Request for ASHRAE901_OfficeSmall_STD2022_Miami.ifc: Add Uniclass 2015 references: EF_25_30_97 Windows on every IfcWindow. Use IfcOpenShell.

First a look at what the model holds.

```python
import ifcopenshell

model = ifcopenshell.open("ASHRAE901_OfficeSmall_STD2022_Miami.ifc")
print(model.schema)
print("classifications:", [c.Name for c in model.by_type("IfcClassification")])
for ifc_class in ("IfcDoor", "IfcRoof", "IfcStair", "IfcWall", "IfcWindow"):
    print(ifc_class, len(model.by_type(ifc_class)))
```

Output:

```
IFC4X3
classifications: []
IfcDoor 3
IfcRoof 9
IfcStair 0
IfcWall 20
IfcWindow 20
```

```python
import ifcopenshell
import ifcopenshell.api.classification

model = ifcopenshell.open("ASHRAE901_OfficeSmall_STD2022_Miami.ifc")

system = ifcopenshell.api.classification.add_classification(model, classification="Uniclass 2015")

codes = {
    "IfcWindow": ("EF_25_30_97", "Windows"),
}
for ifc_class, (code, name) in codes.items():
    products = model.by_type(ifc_class)
    ifcopenshell.api.classification.add_reference(
        model, products=products, classification=system, identification=code, name=name
    )
    print(code, len(products))

model.write("ASHRAE901_OfficeSmall_STD2022_Miami_v2.ifc")
```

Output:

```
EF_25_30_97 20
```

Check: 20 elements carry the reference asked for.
